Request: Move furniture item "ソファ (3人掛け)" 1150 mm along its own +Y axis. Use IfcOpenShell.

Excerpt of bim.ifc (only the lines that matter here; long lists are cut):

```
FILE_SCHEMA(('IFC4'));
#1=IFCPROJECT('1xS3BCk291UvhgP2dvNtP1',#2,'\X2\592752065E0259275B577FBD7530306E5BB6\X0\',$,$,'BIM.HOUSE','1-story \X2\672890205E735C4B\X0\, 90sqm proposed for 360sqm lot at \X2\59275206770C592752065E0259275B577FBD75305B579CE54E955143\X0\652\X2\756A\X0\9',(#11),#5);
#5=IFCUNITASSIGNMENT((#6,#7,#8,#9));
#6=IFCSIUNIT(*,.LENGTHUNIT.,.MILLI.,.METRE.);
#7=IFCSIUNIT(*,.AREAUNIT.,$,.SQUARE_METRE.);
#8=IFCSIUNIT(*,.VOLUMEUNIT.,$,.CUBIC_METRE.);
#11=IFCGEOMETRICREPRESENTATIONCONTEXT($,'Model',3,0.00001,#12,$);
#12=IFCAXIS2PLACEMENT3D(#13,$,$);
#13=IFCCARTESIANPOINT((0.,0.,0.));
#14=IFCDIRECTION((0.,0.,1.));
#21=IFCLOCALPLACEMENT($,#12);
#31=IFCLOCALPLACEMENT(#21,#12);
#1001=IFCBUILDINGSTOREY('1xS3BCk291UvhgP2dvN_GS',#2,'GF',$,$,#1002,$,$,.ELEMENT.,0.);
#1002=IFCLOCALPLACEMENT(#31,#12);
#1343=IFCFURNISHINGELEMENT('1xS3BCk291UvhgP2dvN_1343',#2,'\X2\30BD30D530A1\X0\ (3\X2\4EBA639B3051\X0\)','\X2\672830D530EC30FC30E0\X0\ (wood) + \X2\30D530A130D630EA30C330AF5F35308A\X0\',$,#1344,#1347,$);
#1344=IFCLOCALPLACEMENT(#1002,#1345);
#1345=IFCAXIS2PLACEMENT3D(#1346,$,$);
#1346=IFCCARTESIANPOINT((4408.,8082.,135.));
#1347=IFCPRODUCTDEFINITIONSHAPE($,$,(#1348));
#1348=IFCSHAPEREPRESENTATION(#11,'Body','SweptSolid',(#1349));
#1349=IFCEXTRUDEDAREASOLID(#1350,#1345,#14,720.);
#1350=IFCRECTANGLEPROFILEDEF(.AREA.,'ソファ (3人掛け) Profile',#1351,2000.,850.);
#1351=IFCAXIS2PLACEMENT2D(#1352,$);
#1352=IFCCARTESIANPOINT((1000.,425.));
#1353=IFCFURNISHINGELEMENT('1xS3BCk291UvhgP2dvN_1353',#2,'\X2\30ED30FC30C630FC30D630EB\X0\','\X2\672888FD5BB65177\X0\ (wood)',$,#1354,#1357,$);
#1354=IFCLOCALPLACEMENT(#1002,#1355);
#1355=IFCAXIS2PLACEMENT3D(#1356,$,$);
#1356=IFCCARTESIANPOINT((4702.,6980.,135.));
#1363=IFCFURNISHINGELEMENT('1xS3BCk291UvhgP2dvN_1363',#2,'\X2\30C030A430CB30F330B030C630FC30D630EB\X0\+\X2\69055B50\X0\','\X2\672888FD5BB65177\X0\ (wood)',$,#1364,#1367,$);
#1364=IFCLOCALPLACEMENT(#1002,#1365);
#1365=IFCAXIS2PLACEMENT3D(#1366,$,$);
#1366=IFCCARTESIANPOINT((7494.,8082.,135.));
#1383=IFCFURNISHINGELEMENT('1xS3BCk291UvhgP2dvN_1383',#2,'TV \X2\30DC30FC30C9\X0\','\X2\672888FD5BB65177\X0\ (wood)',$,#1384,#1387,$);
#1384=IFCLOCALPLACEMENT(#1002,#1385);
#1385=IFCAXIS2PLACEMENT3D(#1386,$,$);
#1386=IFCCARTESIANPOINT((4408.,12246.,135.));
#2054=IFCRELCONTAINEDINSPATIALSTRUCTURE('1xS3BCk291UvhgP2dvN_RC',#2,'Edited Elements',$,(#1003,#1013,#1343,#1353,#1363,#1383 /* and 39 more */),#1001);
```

```python
import ifcopenshell
import ifcopenshell.api.geometry
import ifcopenshell.util.placement
import ifcopenshell.util.unit

model = ifcopenshell.open("bim.ifc")
unit_scale = ifcopenshell.util.unit.calculate_unit_scale(model)

item = model.by_id(1343)
matrix = ifcopenshell.util.placement.get_local_placement(item.ObjectPlacement)
matrix[:3, 3] += matrix[:3, 1] * 1.15 / unit_scale
ifcopenshell.api.geometry.edit_object_placement(model, product=item, matrix=matrix, is_si=False)

print(ifcopenshell.util.placement.get_local_placement(item.ObjectPlacement).round(3) + 0.0)

model.write("bim_updated.ifc")
```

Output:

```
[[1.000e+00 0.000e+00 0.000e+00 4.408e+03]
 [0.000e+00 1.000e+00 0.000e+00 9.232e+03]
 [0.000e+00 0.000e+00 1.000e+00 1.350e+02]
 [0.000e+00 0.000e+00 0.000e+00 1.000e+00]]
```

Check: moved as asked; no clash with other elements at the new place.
